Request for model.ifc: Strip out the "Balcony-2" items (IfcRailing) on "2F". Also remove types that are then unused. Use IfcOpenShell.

First a look at what the model holds.

```python
import ifcopenshell
import ifcopenshell.util.element

model = ifcopenshell.open("model.ifc")
print(model.schema)
storey = next(s for s in model.by_type("IfcBuildingStorey") if s.Name == "2F")
railings = [e for e in ifcopenshell.util.element.get_decomposition(storey) if e.is_a("IfcRailing")]
seen = {}
for e in railings:
    element_type = ifcopenshell.util.element.get_type(e)
    name = element_type.Name if element_type not in (None, e) else None
    seen[name] = seen.get(name, 0) + 1
for name, count in sorted(seen.items(), key=str):
    print(count, "x", name)
```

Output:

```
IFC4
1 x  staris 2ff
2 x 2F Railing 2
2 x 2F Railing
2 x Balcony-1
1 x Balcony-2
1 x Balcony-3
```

```python
import ifcopenshell
import ifcopenshell.api.root
import ifcopenshell.util.element

model = ifcopenshell.open("model.ifc")

storey = next(s for s in model.by_type("IfcBuildingStorey") if s.Name == "2F")
railings = [e for e in ifcopenshell.util.element.get_decomposition(storey) if e.is_a("IfcRailing")]
targets = [e for e in railings if (t := ifcopenshell.util.element.get_type(e)) not in (None, e) and t.Name == "Balcony-2"]
types = {ifcopenshell.util.element.get_type(e) for e in targets} - {None, *targets}

for e in targets:
    ifcopenshell.api.root.remove_product(model, product=e)
print(len(targets), "removed")

unused = [t for t in types if not ifcopenshell.util.element.get_types(t)]
for t in unused:
    ifcopenshell.api.root.remove_product(model, product=t)
print(len(unused), "unused types removed")

model.write("model_rev.ifc")
```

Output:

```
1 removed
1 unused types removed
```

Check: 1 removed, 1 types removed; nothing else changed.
